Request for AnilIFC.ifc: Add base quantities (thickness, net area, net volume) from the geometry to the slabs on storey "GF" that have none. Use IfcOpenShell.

First a look at what the model holds.

```python
import ifcopenshell
import ifcopenshell.util.element
import ifcopenshell.util.unit

model = ifcopenshell.open("AnilIFC.ifc")
print(model.schema)
for unit_type in ("LENGTHUNIT", "AREAUNIT", "VOLUMEUNIT"):
    print(unit_type, ifcopenshell.util.unit.calculate_unit_scale(model, unit_type))
storey = next(s for s in model.by_type("IfcBuildingStorey") if s.Name == "GF")
slabs = [e for e in ifcopenshell.util.element.get_decomposition(storey) if e.is_a("IfcSlab")]
for e in sorted(slabs, key=lambda e: e.id()):
    print(e.id(), e.is_a(), e.Name, list(ifcopenshell.util.element.get_psets(e, qtos_only=True)), sep=" | ")
```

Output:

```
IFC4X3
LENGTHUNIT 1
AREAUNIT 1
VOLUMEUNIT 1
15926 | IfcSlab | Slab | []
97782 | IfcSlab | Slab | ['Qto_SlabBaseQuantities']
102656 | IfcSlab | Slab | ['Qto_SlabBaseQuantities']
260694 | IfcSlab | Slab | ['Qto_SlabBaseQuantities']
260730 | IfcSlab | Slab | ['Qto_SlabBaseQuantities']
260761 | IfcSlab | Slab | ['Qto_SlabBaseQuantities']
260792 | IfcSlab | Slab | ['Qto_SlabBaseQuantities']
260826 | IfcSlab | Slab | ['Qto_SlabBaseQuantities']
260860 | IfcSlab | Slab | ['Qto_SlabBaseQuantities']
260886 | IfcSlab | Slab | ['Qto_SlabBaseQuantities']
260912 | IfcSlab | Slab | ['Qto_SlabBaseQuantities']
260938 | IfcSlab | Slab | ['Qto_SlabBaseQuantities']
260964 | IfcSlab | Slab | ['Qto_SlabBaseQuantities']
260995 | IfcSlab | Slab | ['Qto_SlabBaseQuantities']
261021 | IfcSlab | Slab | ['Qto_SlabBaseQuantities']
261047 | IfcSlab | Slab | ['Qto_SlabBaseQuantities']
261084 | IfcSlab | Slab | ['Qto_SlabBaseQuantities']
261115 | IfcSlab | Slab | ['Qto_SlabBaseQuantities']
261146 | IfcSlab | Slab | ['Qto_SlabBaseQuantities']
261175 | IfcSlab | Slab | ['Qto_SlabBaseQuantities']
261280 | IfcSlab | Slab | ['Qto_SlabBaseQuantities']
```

```python
import ifcopenshell
import ifcopenshell.api.pset
import ifcopenshell.geom
import ifcopenshell.util.element
import ifcopenshell.util.shape
import ifcopenshell.util.unit

model = ifcopenshell.open("AnilIFC.ifc")
unit_scale = ifcopenshell.util.unit.calculate_unit_scale(model)
area_scale = ifcopenshell.util.unit.calculate_unit_scale(model, "AREAUNIT")
volume_scale = ifcopenshell.util.unit.calculate_unit_scale(model, "VOLUMEUNIT")
settings = ifcopenshell.geom.settings()

storey = next(s for s in model.by_type("IfcBuildingStorey") if s.Name == "GF")
slabs = [e for e in ifcopenshell.util.element.get_decomposition(storey) if e.is_a("IfcSlab")]

for e in sorted(slabs, key=lambda e: e.id()):
    if ifcopenshell.util.element.get_psets(e, qtos_only=True, should_inherit=False):
        continue
    # Geometry comes back in metres, in the element's own axes.
    shape = ifcopenshell.geom.create_shape(settings, e)
    values = {
        "Width": ifcopenshell.util.shape.get_z(shape.geometry) / unit_scale,
        "NetArea": ifcopenshell.util.shape.get_footprint_area(shape.geometry) / area_scale,
        "NetVolume": ifcopenshell.util.shape.get_volume(shape.geometry) / volume_scale,
    }
    qto = ifcopenshell.api.pset.add_qto(model, product=e, name="Qto_SlabBaseQuantities")
    ifcopenshell.api.pset.edit_qto(model, qto=qto, properties=values)
    print(e.id(), {k: round(v, 3) for k, v in values.items()})

model.write("AnilIFC_updated.ifc")
```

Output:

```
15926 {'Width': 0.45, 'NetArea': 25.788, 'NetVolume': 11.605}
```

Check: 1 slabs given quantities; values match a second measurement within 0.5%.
